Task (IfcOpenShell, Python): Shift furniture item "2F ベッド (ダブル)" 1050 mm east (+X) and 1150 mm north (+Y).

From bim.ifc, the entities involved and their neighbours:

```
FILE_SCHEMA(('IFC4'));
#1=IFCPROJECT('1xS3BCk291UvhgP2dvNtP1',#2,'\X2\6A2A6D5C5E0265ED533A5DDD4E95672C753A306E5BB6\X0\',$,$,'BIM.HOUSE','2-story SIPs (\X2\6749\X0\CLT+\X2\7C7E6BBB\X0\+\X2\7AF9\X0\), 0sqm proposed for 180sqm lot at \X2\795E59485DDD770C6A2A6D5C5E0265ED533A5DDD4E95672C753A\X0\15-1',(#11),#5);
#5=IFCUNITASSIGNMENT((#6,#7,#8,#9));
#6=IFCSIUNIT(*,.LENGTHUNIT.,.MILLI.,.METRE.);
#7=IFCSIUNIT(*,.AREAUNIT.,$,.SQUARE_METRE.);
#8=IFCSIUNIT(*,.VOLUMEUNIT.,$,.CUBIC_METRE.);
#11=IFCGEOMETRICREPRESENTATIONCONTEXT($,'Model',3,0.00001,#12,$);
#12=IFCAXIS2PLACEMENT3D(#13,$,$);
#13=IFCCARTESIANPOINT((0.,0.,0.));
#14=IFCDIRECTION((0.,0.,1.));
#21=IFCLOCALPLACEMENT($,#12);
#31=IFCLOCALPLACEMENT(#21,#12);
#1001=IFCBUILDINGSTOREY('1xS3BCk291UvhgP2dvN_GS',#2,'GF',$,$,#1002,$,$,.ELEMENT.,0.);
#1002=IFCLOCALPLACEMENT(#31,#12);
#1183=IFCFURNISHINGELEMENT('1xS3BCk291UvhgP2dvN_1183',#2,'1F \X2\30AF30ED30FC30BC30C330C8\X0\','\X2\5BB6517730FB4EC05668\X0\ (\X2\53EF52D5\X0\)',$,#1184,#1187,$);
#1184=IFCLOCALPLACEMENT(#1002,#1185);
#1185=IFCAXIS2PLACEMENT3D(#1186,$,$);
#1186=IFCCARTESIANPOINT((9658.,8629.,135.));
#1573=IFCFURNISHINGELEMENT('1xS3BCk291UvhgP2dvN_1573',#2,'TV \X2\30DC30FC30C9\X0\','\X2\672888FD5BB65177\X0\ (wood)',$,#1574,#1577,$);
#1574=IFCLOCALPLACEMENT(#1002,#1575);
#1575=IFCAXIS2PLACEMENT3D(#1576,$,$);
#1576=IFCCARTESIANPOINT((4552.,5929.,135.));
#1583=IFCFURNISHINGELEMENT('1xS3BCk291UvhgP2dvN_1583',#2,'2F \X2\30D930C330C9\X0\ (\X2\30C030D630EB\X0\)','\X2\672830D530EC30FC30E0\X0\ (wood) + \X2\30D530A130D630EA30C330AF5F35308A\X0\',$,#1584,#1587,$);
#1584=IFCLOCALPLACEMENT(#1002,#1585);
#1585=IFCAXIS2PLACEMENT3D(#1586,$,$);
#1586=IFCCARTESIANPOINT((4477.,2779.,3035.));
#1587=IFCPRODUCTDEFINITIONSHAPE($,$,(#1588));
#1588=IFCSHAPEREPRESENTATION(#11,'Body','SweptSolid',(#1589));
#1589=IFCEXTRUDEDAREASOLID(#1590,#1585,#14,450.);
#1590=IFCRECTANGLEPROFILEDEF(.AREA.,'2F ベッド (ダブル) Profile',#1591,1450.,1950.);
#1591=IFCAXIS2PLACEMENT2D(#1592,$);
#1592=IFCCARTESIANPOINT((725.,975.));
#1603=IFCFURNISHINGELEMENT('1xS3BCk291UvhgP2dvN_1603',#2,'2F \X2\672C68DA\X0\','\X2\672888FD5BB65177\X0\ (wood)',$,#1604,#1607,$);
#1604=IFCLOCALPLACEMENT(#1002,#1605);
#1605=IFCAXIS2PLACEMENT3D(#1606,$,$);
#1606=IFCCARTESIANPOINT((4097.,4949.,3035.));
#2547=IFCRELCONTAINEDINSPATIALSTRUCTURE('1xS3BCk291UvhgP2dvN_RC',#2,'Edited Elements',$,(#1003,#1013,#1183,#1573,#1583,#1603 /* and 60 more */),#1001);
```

```python
import ifcopenshell
import ifcopenshell.api.geometry
import ifcopenshell.util.placement
import ifcopenshell.util.unit

model = ifcopenshell.open("bim.ifc")
unit_scale = ifcopenshell.util.unit.calculate_unit_scale(model)

item = model.by_guid("1xS3BCk291UvhgP2dvN_1583")
matrix = ifcopenshell.util.placement.get_local_placement(item.ObjectPlacement)
matrix[0, 3] += 1.05 / unit_scale
matrix[1, 3] += 1.15 / unit_scale
ifcopenshell.api.geometry.edit_object_placement(model, product=item, matrix=matrix, is_si=False)

print(ifcopenshell.util.placement.get_local_placement(item.ObjectPlacement).round(3) + 0.0)

model.write("bim_v2.ifc")
```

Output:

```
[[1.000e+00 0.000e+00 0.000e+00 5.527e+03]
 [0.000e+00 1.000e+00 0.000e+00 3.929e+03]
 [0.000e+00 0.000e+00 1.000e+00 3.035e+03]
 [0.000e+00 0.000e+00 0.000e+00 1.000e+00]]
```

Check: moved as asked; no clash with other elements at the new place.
